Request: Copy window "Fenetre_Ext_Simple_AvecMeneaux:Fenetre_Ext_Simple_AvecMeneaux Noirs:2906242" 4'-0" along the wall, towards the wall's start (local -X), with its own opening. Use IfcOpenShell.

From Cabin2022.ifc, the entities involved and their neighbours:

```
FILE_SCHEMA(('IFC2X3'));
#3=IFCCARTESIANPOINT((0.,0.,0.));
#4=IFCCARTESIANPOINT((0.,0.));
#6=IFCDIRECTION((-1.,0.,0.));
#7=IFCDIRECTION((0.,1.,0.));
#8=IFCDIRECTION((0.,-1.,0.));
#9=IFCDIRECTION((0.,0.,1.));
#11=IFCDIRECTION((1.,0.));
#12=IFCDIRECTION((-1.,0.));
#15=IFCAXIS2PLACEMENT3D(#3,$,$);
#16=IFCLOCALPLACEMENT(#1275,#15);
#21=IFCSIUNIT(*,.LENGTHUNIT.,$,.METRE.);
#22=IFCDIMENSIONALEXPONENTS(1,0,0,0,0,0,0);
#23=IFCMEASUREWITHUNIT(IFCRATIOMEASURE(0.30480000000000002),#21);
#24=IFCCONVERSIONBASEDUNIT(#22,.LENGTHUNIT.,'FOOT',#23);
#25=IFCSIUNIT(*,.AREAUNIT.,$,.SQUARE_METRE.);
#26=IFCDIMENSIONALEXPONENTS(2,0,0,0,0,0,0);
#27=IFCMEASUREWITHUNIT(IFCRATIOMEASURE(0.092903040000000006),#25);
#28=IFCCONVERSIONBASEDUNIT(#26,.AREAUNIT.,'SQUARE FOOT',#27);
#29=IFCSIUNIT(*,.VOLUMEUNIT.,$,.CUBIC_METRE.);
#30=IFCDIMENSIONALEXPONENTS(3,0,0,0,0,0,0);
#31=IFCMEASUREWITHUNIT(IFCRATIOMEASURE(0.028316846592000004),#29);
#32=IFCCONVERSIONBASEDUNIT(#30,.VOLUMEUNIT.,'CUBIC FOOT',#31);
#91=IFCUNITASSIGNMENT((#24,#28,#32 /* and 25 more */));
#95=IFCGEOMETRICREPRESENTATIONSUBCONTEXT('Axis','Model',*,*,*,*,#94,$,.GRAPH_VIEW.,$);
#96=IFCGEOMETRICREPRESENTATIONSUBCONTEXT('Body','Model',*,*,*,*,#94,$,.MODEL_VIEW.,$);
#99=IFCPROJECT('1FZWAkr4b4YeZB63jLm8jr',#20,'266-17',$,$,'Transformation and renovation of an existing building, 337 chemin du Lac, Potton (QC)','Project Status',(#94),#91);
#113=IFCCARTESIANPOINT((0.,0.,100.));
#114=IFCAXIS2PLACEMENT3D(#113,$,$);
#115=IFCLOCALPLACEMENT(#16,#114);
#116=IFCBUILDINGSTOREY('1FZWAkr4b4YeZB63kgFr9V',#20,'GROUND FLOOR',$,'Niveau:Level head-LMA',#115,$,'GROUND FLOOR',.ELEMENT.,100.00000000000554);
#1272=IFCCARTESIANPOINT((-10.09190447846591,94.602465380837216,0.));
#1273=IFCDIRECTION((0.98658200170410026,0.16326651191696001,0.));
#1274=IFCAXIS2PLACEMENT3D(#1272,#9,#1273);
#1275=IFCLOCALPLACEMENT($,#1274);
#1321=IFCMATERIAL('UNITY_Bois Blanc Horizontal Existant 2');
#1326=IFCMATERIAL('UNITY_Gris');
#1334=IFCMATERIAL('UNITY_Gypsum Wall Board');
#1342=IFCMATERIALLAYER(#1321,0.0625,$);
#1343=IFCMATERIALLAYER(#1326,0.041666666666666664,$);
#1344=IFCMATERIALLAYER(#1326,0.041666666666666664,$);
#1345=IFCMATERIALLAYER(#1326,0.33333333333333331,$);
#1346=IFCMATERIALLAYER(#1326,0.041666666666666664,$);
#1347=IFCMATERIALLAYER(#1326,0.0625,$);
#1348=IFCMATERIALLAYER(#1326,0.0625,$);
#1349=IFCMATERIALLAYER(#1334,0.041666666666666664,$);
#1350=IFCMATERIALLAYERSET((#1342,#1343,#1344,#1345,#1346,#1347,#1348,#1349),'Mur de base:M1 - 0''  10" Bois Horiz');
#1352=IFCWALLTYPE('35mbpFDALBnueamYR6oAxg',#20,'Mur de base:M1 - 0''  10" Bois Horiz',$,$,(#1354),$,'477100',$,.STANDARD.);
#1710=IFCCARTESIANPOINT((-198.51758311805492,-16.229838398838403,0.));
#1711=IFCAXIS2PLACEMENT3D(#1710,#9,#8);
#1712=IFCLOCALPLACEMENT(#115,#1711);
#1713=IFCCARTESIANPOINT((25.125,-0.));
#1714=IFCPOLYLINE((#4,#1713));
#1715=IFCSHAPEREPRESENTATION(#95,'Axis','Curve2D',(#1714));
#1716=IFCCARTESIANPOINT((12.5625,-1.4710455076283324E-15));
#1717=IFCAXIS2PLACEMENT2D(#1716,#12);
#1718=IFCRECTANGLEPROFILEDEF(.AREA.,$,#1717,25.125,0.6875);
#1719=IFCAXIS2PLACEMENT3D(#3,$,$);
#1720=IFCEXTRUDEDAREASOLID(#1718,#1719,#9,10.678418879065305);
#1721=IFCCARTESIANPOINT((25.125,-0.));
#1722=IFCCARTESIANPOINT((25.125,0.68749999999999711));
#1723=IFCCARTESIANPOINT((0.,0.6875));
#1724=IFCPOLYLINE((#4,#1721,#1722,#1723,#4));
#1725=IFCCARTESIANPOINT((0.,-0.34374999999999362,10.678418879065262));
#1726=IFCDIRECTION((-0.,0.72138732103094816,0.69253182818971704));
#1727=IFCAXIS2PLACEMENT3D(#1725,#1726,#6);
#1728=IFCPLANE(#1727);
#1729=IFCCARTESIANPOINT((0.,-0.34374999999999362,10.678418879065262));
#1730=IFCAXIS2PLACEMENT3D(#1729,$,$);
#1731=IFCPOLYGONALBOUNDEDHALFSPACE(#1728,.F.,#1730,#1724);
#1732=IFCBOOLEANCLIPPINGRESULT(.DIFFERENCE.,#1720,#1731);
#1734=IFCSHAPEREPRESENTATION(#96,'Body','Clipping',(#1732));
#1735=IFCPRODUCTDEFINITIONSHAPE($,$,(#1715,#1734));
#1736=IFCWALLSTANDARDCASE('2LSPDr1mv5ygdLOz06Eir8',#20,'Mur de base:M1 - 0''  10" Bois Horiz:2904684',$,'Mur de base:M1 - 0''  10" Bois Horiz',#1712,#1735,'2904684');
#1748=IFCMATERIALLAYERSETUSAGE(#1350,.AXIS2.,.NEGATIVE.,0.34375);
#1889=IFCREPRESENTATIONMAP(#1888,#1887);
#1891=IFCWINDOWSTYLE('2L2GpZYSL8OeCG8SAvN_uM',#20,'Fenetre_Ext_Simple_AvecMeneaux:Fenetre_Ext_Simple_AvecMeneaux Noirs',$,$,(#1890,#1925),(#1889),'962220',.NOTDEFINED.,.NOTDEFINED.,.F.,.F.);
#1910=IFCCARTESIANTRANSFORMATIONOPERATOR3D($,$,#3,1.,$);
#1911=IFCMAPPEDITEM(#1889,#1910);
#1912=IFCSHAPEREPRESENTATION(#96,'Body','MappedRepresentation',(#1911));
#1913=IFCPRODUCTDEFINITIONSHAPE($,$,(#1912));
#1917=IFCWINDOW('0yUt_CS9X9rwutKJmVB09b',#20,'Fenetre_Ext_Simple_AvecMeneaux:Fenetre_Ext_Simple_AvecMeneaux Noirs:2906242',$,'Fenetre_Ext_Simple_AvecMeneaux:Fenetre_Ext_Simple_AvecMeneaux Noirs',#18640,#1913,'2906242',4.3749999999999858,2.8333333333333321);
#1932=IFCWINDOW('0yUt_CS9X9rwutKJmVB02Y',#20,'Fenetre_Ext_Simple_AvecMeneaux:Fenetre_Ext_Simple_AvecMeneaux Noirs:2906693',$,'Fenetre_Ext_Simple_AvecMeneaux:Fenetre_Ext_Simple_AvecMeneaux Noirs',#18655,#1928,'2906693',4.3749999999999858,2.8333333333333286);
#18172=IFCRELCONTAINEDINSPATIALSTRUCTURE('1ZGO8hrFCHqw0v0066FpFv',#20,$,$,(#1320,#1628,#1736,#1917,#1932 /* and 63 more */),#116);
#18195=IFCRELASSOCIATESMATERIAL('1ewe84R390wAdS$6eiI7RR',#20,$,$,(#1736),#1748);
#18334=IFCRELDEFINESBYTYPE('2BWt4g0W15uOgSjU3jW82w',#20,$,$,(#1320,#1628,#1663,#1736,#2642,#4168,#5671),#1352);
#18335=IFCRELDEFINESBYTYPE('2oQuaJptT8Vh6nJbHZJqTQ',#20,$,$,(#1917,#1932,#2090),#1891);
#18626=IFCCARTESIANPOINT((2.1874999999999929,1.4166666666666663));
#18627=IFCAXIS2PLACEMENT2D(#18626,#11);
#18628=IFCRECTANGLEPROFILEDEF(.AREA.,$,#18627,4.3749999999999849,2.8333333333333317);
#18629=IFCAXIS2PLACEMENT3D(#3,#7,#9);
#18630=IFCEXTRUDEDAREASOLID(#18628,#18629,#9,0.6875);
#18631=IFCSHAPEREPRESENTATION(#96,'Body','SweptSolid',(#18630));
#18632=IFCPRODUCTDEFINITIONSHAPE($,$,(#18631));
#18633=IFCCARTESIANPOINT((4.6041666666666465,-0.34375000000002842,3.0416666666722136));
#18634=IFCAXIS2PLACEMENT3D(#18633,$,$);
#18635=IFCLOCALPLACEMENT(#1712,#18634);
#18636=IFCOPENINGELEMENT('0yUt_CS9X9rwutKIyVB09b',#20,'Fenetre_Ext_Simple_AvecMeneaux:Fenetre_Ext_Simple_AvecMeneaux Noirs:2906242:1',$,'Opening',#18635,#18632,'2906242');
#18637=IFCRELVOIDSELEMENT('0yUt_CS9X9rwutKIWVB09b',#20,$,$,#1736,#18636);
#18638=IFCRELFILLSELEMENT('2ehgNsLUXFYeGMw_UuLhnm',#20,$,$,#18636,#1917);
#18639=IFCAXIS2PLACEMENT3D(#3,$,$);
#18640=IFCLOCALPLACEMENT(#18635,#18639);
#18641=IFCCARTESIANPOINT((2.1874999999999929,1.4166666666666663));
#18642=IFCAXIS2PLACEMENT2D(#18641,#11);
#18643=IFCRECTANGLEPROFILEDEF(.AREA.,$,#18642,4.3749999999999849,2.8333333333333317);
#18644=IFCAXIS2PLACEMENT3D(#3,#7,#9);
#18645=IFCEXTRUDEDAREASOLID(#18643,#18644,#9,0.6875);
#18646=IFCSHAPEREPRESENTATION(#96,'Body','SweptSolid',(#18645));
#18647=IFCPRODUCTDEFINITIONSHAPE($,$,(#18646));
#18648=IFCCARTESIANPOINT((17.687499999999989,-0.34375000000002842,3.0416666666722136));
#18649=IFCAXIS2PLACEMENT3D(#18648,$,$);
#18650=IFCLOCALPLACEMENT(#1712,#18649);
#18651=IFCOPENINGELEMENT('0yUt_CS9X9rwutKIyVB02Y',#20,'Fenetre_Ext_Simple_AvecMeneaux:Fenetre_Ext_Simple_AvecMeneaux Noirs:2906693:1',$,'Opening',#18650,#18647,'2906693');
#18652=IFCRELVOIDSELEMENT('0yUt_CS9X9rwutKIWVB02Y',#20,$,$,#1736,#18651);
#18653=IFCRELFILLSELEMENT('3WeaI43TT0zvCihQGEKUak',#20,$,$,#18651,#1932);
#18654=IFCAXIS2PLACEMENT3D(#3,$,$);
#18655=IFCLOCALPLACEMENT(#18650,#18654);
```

```python
import ifcopenshell
import ifcopenshell.api.feature
import ifcopenshell.api.geometry
import ifcopenshell.api.root
import ifcopenshell.geom
import ifcopenshell.util.element
import ifcopenshell.util.placement
import ifcopenshell.util.shape
import ifcopenshell.util.unit

model = ifcopenshell.open("Cabin2022.ifc")
unit_scale = ifcopenshell.util.unit.calculate_unit_scale(model)
settings = ifcopenshell.geom.settings()


def volume(element):
    """Net volume in cubic metres, openings subtracted."""
    shape = ifcopenshell.geom.create_shape(settings, element)
    return ifcopenshell.util.shape.get_volume(shape.geometry)


def reuse_history(source, copy):
    """copy_class also copies each property set's owner history, people and application; keep the originals."""
    for rel in copy.IsDefinedBy:
        if rel.is_a("IfcRelDefinesByProperties") and (history := rel.RelatingPropertyDefinition.OwnerHistory):
            rel.RelatingPropertyDefinition.OwnerHistory = source.OwnerHistory
            ifcopenshell.util.element.remove_deep2(model, history)


window = model.by_id(1917)
opening = window.FillsVoids[0].RelatingOpeningElement
wall = opening.VoidsElements[0].RelatingBuildingElement
before = volume(wall)
shift = ifcopenshell.util.placement.get_local_placement(wall.ObjectPlacement)[:3, 0] * -48 * 0.0254 / unit_scale

# copy_class copies the void relationship, type, container and properties, but no geometry.
new_opening = ifcopenshell.api.root.copy_class(model, product=opening)
new_opening.Representation = ifcopenshell.util.element.copy_deep(
    model, opening.Representation, exclude=["IfcGeometricRepresentationContext", "IfcRepresentationMap"]
)
new_opening.Name = "Fenetre_Ext_Simple_AvecMeneaux:Fenetre_Ext_Simple_AvecMeneaux Noirs"
new_opening.Tag = None
new_window = ifcopenshell.api.root.copy_class(model, product=window)
new_window.Representation = ifcopenshell.util.element.copy_deep(
    model, window.Representation, exclude=["IfcGeometricRepresentationContext", "IfcRepresentationMap"]
)
new_window.Name = "Fenetre_Ext_Simple_AvecMeneaux:Fenetre_Ext_Simple_AvecMeneaux Noirs"
new_window.Tag = None
reuse_history(window, new_window)
fills = ifcopenshell.api.feature.add_filling(model, opening=new_opening, element=new_window)
fills.OwnerHistory = new_window.OwnerHistory  # required in IFC2X3

for old, new in ((opening, new_opening), (window, new_window)):
    matrix = ifcopenshell.util.placement.get_local_placement(old.ObjectPlacement)
    matrix[:3, 3] += shift
    ifcopenshell.api.geometry.edit_object_placement(model, product=new, matrix=matrix, is_si=False)

after = volume(wall)

print(f"wall volume {before:.3f} -> {after:.3f} m3")

model.write("Cabin2022_updated.ifc")
```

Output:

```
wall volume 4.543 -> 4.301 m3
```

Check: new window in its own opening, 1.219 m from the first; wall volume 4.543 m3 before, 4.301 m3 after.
